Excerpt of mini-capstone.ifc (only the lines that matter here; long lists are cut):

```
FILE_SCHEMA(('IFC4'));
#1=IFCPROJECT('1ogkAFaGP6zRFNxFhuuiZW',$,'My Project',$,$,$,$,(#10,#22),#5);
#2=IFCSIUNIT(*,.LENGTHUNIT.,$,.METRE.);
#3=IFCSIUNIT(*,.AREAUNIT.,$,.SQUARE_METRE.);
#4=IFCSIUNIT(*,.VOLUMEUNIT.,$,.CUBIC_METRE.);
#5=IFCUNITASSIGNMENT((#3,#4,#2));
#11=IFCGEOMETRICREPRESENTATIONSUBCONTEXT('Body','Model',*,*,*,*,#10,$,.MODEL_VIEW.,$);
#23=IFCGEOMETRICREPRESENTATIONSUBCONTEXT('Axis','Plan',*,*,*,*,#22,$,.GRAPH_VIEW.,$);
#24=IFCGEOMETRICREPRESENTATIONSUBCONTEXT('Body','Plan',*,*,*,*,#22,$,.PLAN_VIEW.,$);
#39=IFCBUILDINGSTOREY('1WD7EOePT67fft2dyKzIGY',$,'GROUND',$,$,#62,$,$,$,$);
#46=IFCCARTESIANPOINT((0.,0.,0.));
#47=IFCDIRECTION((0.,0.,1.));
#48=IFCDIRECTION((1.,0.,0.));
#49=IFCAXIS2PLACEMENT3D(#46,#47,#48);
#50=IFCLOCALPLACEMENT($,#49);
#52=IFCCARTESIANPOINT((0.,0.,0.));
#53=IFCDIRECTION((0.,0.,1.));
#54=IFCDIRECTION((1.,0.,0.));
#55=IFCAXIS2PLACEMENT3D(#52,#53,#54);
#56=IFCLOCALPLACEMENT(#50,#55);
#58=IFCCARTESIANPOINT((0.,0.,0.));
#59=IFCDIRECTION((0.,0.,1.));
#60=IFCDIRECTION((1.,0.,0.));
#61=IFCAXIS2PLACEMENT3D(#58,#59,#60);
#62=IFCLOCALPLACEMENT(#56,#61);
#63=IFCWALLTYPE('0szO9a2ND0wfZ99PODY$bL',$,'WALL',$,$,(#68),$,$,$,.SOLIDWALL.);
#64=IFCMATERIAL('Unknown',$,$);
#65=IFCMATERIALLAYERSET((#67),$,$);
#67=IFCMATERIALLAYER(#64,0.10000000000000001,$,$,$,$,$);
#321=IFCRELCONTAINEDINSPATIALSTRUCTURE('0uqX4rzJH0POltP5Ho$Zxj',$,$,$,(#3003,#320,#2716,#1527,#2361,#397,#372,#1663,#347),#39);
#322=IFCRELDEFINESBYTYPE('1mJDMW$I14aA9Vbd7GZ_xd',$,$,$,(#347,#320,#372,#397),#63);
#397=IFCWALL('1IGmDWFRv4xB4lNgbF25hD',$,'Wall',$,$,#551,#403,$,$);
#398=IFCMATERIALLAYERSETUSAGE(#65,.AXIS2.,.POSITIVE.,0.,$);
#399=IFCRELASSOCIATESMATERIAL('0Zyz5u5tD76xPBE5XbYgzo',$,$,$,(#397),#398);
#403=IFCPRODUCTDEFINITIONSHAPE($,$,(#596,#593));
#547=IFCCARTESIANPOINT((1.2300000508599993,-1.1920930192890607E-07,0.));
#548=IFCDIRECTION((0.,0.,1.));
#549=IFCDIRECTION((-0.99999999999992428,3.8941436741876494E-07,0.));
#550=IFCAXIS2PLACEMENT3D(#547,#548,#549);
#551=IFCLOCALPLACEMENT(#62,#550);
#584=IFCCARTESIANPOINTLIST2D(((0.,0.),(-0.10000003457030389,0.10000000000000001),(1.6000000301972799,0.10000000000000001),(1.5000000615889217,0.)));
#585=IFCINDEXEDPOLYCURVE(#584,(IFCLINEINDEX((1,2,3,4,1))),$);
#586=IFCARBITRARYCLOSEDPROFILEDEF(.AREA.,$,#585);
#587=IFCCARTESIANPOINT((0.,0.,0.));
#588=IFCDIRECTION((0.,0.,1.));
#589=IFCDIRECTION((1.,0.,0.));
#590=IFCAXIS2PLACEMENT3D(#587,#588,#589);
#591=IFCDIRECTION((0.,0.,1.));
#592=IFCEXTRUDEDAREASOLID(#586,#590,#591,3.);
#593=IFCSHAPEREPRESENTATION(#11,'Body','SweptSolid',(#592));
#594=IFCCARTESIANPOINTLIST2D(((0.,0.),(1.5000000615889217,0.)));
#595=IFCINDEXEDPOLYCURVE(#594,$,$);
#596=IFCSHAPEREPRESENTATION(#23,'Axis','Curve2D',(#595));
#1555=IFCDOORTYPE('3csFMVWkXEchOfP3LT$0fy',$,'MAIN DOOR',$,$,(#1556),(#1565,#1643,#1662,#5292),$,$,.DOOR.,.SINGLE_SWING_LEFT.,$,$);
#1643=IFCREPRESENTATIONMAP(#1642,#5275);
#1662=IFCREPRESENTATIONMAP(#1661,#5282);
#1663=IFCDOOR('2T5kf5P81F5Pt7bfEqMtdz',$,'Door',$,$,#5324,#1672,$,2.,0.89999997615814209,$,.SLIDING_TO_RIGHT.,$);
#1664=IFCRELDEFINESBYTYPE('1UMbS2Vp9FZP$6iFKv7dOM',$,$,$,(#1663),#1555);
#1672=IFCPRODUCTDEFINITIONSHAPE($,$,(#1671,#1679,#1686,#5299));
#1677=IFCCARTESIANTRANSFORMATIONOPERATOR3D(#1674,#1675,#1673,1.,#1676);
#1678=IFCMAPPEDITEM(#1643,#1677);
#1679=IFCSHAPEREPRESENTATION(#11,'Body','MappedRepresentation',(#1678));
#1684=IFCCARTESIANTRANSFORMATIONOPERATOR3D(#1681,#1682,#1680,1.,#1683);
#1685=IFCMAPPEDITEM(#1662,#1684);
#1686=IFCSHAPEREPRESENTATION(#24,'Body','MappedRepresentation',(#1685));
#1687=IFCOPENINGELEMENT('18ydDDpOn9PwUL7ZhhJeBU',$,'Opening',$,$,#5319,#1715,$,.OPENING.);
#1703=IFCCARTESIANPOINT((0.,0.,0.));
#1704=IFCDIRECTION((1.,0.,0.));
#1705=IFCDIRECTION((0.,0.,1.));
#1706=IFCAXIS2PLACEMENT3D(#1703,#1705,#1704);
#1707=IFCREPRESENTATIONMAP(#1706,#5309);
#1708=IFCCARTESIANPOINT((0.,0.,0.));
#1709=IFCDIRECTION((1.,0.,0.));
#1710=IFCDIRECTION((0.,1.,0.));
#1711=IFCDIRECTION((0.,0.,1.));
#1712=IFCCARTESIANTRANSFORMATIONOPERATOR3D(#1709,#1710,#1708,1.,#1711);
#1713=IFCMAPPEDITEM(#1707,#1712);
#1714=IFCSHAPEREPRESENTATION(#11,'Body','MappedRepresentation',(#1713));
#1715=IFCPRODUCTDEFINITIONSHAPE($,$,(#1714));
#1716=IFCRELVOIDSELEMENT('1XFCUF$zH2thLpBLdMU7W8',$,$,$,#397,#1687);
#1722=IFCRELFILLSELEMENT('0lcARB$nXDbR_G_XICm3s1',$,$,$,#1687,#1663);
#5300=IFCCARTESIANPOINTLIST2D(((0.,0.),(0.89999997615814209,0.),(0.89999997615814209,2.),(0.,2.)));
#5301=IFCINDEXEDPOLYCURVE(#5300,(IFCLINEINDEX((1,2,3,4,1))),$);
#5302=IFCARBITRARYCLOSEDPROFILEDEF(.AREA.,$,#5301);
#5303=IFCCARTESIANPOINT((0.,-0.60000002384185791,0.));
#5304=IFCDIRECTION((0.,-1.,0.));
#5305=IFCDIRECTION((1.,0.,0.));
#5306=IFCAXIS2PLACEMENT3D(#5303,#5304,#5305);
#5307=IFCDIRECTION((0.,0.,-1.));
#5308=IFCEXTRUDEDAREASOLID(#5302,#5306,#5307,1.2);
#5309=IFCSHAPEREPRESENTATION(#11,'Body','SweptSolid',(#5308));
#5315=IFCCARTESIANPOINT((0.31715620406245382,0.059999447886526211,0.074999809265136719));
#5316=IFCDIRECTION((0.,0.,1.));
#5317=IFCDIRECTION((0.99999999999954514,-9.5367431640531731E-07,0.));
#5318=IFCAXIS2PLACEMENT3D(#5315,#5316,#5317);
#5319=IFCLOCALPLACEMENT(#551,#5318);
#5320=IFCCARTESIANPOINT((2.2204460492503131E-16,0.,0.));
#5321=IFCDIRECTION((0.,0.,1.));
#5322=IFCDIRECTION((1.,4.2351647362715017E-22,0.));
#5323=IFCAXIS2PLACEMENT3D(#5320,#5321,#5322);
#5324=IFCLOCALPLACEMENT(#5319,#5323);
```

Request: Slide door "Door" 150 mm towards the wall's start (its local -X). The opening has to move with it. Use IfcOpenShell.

```python
import ifcopenshell
import ifcopenshell.api.geometry
import ifcopenshell.util.placement

model = ifcopenshell.open("mini-capstone.ifc")

door = model.by_guid("2T5kf5P81F5Pt7bfEqMtdz")
opening = door.FillsVoids[0].RelatingOpeningElement
wall = opening.VoidsElements[0].RelatingBuildingElement

wall_matrix = ifcopenshell.util.placement.get_local_placement(wall.ObjectPlacement)
shift = wall_matrix[:3, 0] * -0.15
before = ifcopenshell.util.placement.get_local_placement(door.ObjectPlacement)[:3, 3].copy()

# The door is placed relative to its opening, so it follows when the opening moves.
matrix = ifcopenshell.util.placement.get_local_placement(opening.ObjectPlacement)
matrix[:3, 3] += shift
ifcopenshell.api.geometry.edit_object_placement(
    model, product=opening, matrix=matrix, is_si=False, should_transform_children=True
)

after = ifcopenshell.util.placement.get_local_placement(door.ObjectPlacement)[:3, 3]
print("door moved by", (after - before).round(3) + 0.0)

model.write("mini-capstone_rev.ifc")
```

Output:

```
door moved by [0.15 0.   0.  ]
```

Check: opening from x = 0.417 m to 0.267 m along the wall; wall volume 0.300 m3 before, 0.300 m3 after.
